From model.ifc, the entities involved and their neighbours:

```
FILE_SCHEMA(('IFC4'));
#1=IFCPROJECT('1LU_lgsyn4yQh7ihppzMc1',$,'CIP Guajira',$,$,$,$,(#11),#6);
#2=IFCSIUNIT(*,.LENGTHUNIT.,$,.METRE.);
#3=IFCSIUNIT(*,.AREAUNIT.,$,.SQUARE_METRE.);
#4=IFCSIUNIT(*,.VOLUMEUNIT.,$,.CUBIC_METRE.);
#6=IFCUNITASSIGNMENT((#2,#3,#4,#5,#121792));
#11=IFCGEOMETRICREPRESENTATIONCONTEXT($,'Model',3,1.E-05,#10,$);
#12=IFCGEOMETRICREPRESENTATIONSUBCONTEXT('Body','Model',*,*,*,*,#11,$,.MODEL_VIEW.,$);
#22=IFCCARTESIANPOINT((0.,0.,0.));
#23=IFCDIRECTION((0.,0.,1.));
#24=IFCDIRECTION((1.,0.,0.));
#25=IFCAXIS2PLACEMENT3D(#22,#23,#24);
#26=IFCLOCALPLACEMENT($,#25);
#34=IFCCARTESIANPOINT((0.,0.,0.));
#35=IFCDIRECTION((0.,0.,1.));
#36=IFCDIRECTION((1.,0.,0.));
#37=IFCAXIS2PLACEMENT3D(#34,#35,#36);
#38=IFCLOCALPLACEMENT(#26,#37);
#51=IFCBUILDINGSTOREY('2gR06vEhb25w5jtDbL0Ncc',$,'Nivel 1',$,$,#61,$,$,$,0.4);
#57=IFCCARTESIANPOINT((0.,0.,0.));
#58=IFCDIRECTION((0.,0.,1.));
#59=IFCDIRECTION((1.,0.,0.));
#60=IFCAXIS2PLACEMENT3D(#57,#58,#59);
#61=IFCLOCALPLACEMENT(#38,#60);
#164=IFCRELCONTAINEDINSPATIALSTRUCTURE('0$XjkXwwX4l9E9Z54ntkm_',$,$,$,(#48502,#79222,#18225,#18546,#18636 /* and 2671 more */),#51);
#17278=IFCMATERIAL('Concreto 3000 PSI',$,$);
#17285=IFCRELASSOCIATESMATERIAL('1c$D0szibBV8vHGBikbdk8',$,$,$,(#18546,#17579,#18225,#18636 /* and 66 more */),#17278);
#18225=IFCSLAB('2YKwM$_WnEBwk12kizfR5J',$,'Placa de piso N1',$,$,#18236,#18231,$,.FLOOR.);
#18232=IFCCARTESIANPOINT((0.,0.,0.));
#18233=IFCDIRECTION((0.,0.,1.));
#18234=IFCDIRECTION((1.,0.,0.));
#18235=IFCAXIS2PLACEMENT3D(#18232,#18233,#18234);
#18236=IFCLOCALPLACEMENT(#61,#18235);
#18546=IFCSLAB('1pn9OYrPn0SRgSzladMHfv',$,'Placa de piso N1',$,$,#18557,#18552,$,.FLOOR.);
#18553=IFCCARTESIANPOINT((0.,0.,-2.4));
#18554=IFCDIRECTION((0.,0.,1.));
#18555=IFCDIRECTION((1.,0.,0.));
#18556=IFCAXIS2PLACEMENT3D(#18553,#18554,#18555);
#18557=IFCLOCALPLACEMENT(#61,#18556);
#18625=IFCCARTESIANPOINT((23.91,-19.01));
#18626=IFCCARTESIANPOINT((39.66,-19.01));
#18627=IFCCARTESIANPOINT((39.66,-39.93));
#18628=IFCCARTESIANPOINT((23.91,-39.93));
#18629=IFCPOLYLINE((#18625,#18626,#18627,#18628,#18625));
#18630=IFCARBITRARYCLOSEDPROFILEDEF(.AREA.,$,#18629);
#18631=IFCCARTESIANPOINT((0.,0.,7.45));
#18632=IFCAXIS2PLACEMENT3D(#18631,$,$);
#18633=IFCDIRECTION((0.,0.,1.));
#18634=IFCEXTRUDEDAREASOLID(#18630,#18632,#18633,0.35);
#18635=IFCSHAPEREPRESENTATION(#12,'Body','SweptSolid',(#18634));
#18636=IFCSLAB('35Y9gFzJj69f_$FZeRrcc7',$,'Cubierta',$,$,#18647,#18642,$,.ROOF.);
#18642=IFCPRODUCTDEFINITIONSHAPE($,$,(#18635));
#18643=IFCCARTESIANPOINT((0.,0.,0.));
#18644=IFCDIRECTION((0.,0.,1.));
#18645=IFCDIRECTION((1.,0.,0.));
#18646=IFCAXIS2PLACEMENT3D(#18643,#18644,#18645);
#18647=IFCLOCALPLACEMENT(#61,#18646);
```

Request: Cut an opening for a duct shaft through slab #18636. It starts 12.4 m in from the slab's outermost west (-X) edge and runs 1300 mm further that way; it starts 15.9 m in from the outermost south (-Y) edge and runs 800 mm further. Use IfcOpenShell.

```python
import numpy as np
import ifcopenshell
import ifcopenshell.api.feature
import ifcopenshell.api.geometry
import ifcopenshell.api.root
import ifcopenshell.geom
import ifcopenshell.util.placement
import ifcopenshell.util.representation
import ifcopenshell.util.shape
import ifcopenshell.util.unit

model = ifcopenshell.open("model.ifc")
unit_scale = ifcopenshell.util.unit.calculate_unit_scale(model)
settings = ifcopenshell.geom.settings()


def volume(element):
    """Net volume in cubic metres, openings subtracted."""
    shape = ifcopenshell.geom.create_shape(settings, element)
    return ifcopenshell.util.shape.get_volume(shape.geometry)


slab = model.by_guid("35Y9gFzJj69f_$FZeRrcc7")
before = volume(slab)

# Extent in the slab's own axes, in metres. The edges named are its -X and -Y sides.
slab_shape = ifcopenshell.geom.create_shape(settings, slab)
vertices = ifcopenshell.util.shape.get_vertices(slab_shape.geometry)
x_min, y_min, bottom = vertices.min(axis=0)
top = vertices[:, 2].max()

opening = ifcopenshell.api.root.create_entity(model, ifc_class="IfcOpeningElement", name="Duct shaft opening", predefined_type="OPENING")
context = ifcopenshell.util.representation.get_context(model, "Model", "Body", "MODEL_VIEW")
width, depth = 1.3, 0.8
outline = [(0.0, 0.0), (width, 0.0), (width, depth), (0.0, depth), (0.0, 0.0)]
# Overshoot both faces by 50 mm so the cut is clean.
shape = ifcopenshell.api.geometry.add_slab_representation(
    model, context=context, depth=top - bottom + 0.1, polyline=outline
)
ifcopenshell.api.geometry.assign_representation(model, product=opening, representation=shape)

matrix = ifcopenshell.util.placement.get_local_placement(slab.ObjectPlacement)
matrix[:, 3] = matrix @ np.append(np.array([x_min + 12.4, y_min + 15.9, bottom - 0.05]) / unit_scale, 1.0)
ifcopenshell.api.geometry.edit_object_placement(model, product=opening, matrix=matrix, is_si=False)
ifcopenshell.api.feature.add_feature(model, feature=opening, element=slab)

after = volume(slab)

print(f"slab volume {before:.3f} -> {after:.3f} m3")

model.write("model_edited.ifc")
```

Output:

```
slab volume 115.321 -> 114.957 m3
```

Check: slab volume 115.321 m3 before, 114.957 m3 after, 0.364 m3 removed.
